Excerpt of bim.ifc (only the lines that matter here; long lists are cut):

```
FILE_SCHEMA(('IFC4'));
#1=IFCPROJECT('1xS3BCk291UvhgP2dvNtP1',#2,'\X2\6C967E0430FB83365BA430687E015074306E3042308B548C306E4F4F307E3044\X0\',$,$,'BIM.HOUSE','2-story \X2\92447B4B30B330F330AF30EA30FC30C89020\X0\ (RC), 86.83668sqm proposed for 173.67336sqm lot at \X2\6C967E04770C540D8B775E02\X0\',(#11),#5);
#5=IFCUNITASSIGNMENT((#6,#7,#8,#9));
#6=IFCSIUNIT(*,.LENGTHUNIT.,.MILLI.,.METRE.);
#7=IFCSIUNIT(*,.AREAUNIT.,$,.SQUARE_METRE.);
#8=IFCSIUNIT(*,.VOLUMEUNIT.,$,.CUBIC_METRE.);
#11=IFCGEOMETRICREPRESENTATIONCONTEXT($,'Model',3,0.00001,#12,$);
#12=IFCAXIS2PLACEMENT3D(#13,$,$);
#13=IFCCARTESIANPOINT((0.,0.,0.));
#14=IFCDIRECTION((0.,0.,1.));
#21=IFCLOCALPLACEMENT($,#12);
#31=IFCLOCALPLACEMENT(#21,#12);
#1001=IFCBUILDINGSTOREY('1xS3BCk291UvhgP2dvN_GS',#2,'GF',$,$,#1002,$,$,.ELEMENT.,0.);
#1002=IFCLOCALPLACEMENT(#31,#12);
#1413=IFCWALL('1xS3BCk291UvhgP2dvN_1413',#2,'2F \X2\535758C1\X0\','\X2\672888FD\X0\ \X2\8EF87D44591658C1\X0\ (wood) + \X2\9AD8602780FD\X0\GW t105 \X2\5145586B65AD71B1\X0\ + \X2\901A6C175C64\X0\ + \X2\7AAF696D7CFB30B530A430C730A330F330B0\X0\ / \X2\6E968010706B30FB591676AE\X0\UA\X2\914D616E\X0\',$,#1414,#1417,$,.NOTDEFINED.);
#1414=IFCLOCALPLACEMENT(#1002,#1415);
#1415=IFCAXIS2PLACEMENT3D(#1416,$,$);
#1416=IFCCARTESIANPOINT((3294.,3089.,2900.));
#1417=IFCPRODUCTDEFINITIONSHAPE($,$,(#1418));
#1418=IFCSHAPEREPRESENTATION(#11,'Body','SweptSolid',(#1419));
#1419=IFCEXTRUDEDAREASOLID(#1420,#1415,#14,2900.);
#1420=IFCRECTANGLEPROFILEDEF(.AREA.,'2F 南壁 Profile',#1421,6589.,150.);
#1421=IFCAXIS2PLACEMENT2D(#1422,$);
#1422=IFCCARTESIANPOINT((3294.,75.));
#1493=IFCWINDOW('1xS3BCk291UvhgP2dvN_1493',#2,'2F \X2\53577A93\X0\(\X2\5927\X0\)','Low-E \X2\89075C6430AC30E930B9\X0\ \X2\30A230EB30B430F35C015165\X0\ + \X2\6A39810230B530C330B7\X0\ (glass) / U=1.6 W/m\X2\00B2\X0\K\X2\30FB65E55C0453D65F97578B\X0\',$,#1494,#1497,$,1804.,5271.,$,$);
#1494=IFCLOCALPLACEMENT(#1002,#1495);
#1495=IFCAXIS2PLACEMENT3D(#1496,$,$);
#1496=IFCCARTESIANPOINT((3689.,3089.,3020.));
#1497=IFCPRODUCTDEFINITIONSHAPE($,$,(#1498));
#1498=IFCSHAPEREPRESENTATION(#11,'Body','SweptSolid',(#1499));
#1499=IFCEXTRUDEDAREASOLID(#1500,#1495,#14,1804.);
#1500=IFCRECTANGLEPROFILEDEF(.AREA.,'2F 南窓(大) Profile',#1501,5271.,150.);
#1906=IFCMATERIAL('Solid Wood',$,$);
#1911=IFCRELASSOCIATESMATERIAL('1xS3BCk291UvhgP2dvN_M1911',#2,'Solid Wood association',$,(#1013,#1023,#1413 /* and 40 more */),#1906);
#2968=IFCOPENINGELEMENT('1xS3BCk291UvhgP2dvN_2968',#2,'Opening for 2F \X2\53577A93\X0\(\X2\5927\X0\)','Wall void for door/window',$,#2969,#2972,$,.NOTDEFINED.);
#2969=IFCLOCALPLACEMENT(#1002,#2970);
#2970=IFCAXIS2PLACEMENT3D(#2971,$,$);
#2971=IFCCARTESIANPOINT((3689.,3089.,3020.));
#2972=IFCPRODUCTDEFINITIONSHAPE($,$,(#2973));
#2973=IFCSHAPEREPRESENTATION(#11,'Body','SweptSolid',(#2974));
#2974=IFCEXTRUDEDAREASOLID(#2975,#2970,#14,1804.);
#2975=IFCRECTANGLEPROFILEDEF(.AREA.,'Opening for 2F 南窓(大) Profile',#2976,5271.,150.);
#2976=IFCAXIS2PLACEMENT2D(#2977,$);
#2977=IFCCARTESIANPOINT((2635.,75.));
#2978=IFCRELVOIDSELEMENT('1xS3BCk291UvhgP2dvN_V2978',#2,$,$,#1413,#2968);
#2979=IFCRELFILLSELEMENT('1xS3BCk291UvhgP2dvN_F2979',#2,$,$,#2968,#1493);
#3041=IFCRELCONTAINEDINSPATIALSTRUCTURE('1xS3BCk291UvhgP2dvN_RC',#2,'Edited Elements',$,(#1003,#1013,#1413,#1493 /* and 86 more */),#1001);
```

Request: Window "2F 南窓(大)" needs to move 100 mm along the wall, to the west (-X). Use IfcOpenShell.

```python
import ifcopenshell
import ifcopenshell.api.geometry
import ifcopenshell.util.placement
import ifcopenshell.util.unit

model = ifcopenshell.open("bim.ifc")
unit_scale = ifcopenshell.util.unit.calculate_unit_scale(model)

window = model.by_guid("1xS3BCk291UvhgP2dvN_1493")
opening = window.FillsVoids[0].RelatingOpeningElement
wall = opening.VoidsElements[0].RelatingBuildingElement

wall_matrix = ifcopenshell.util.placement.get_local_placement(wall.ObjectPlacement)
shift = wall_matrix[:3, 0] * -0.1 / unit_scale
before = ifcopenshell.util.placement.get_local_placement(window.ObjectPlacement)[:3, 3].copy()

# The window is not placed relative to its opening, so move both.
for product in (opening, window):
    matrix = ifcopenshell.util.placement.get_local_placement(product.ObjectPlacement)
    matrix[:3, 3] += shift
    ifcopenshell.api.geometry.edit_object_placement(model, product=product, matrix=matrix, is_si=False)

after = ifcopenshell.util.placement.get_local_placement(window.ObjectPlacement)[:3, 3]
print("window moved by", (after - before).round(3) + 0.0)

model.write("bim_rev.ifc")
```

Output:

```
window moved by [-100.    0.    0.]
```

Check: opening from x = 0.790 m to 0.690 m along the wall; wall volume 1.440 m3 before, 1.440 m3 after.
